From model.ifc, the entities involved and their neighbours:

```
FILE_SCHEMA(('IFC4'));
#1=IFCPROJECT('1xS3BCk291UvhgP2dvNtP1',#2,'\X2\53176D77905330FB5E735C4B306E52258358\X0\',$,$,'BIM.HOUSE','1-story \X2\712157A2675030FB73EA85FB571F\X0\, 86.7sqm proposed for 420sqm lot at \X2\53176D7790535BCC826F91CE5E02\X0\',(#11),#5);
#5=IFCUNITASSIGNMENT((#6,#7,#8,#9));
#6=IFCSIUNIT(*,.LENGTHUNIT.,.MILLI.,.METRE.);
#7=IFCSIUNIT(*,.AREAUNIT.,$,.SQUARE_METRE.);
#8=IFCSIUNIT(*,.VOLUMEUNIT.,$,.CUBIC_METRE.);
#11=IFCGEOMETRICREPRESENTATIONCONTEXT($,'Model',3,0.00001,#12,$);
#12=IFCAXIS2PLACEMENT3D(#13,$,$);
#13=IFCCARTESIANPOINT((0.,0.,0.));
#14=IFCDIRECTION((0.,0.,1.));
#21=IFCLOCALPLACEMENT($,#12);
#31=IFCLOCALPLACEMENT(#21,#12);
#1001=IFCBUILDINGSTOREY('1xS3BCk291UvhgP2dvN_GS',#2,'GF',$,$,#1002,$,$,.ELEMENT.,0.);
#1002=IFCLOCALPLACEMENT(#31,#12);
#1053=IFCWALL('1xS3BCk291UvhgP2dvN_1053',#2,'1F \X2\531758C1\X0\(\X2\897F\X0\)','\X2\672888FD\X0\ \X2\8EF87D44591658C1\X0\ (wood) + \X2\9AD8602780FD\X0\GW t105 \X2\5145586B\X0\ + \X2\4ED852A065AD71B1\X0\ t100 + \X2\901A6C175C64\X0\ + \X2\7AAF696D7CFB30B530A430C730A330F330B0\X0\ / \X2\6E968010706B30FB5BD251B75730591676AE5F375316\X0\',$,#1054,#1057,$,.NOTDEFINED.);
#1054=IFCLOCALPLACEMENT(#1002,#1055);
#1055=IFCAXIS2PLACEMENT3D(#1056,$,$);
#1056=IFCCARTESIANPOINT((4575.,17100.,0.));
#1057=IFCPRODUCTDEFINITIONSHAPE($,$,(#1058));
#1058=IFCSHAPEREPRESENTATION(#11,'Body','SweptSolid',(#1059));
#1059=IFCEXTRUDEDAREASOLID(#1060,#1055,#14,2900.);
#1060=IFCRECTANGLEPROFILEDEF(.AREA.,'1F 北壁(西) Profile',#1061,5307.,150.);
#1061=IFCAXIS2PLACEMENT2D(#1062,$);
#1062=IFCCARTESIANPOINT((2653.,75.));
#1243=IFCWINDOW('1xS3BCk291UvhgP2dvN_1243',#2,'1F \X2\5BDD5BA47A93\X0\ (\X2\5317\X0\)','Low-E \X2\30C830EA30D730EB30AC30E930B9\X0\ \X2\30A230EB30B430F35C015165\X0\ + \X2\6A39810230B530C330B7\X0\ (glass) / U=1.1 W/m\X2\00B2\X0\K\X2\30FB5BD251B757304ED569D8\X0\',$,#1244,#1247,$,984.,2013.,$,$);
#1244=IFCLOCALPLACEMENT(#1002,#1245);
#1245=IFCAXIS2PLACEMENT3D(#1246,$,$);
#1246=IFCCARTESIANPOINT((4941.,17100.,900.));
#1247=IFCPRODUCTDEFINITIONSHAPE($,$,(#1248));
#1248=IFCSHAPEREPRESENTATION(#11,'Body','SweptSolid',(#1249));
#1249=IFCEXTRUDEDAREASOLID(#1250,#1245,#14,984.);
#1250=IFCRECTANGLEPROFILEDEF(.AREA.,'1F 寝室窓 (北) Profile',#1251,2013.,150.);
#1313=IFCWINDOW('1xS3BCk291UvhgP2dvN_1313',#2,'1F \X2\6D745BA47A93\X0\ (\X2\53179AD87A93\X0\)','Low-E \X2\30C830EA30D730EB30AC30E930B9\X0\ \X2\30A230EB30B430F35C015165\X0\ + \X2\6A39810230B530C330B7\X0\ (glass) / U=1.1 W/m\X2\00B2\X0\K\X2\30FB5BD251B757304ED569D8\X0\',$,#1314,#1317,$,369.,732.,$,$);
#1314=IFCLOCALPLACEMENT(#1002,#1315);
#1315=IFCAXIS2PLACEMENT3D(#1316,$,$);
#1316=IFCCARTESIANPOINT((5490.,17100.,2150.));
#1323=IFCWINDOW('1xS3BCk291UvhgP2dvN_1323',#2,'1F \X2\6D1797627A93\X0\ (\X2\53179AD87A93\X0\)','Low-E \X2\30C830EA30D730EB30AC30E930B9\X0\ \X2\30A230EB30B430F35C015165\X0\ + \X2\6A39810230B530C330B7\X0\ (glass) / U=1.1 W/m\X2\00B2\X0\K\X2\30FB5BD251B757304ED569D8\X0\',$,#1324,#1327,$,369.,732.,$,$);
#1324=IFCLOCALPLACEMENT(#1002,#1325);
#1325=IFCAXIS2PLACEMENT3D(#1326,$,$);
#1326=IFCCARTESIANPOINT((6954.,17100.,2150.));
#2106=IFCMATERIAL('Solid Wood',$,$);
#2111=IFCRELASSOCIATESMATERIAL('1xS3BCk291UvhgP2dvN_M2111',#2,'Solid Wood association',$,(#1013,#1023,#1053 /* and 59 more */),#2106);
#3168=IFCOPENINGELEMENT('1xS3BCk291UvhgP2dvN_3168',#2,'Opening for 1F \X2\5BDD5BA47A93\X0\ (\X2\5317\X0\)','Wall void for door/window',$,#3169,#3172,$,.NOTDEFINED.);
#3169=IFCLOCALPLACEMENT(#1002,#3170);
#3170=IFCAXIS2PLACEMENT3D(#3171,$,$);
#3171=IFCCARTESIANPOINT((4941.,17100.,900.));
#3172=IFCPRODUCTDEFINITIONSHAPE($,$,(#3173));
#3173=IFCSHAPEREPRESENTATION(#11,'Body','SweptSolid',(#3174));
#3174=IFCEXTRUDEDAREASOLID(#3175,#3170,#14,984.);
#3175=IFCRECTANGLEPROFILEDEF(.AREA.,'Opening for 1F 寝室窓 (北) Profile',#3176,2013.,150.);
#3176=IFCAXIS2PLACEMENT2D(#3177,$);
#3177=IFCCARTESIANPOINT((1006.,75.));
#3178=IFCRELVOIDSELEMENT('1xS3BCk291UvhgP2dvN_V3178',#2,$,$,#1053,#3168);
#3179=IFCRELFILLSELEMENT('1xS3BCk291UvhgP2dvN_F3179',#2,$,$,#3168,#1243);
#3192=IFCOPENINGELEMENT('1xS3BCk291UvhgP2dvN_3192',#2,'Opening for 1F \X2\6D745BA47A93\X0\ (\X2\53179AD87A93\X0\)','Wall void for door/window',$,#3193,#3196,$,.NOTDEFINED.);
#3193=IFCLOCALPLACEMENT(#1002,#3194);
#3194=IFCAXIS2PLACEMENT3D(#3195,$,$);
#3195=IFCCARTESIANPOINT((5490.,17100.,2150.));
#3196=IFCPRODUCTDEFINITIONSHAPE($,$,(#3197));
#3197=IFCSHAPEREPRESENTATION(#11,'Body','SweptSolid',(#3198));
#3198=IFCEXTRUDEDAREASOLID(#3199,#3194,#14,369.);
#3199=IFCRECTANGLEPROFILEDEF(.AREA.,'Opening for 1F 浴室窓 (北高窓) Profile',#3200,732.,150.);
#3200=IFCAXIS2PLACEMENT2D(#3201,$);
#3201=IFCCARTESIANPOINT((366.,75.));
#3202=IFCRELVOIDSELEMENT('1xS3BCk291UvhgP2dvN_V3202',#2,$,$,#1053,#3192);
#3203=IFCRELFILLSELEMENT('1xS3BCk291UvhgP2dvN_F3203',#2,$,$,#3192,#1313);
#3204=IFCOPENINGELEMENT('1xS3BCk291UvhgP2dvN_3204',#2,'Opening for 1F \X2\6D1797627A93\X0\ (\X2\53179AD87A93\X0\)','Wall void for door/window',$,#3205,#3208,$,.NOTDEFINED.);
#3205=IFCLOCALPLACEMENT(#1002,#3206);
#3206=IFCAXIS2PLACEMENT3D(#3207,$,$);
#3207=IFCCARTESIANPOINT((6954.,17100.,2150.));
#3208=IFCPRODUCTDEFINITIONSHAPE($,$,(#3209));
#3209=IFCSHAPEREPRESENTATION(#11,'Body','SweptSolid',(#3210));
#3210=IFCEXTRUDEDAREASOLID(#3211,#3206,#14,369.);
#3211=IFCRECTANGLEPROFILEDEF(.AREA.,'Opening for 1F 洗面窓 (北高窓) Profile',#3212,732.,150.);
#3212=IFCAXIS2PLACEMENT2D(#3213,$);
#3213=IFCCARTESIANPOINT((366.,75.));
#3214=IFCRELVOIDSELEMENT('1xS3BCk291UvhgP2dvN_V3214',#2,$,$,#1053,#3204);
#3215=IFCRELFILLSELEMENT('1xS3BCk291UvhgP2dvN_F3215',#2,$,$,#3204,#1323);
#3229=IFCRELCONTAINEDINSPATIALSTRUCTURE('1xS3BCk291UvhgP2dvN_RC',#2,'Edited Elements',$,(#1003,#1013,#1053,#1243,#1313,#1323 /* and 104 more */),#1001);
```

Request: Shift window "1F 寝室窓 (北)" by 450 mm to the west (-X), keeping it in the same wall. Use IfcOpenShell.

```python
import ifcopenshell
import ifcopenshell.api.geometry
import ifcopenshell.util.placement

model = ifcopenshell.open("model.ifc")

window = model.by_guid("1xS3BCk291UvhgP2dvN_1243")
opening = window.FillsVoids[0].RelatingOpeningElement
wall = opening.VoidsElements[0].RelatingBuildingElement

wall_matrix = ifcopenshell.util.placement.get_local_placement(wall.ObjectPlacement)
shift = wall_matrix[:3, 0] * -450.0
before = ifcopenshell.util.placement.get_local_placement(window.ObjectPlacement)[:3, 3].copy()

# The window is not placed relative to its opening, so move both.
for product in (opening, window):
    matrix = ifcopenshell.util.placement.get_local_placement(product.ObjectPlacement)
    matrix[:3, 3] += shift
    ifcopenshell.api.geometry.edit_object_placement(model, product=product, matrix=matrix, is_si=False)

after = ifcopenshell.util.placement.get_local_placement(window.ObjectPlacement)[:3, 3]
print("window moved by", (after - before).round(3) + 0.0)

model.write("model_v2.ifc")
```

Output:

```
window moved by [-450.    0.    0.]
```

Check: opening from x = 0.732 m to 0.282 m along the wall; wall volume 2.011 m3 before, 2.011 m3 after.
